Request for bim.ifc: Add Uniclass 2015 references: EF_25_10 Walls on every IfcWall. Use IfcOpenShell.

First a look at what the model holds.

```python
import ifcopenshell

model = ifcopenshell.open("bim.ifc")
print(model.schema)
print("classifications:", [c.Name for c in model.by_type("IfcClassification")])
for ifc_class in ("IfcDoor", "IfcRoof", "IfcStair", "IfcWall", "IfcWindow"):
    print(ifc_class, len(model.by_type(ifc_class)))
```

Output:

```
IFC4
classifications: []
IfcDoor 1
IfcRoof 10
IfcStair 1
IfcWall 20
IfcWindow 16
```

```python
import ifcopenshell
import ifcopenshell.api.classification

model = ifcopenshell.open("bim.ifc")

system = ifcopenshell.api.classification.add_classification(model, classification="Uniclass 2015")

codes = {
    "IfcWall": ("EF_25_10", "Walls"),
}
for ifc_class, (code, name) in codes.items():
    products = model.by_type(ifc_class)
    ifcopenshell.api.classification.add_reference(
        model, products=products, classification=system, identification=code, name=name
    )
    print(code, len(products))

model.write("bim_v2.ifc")
```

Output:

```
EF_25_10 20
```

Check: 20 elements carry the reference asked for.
